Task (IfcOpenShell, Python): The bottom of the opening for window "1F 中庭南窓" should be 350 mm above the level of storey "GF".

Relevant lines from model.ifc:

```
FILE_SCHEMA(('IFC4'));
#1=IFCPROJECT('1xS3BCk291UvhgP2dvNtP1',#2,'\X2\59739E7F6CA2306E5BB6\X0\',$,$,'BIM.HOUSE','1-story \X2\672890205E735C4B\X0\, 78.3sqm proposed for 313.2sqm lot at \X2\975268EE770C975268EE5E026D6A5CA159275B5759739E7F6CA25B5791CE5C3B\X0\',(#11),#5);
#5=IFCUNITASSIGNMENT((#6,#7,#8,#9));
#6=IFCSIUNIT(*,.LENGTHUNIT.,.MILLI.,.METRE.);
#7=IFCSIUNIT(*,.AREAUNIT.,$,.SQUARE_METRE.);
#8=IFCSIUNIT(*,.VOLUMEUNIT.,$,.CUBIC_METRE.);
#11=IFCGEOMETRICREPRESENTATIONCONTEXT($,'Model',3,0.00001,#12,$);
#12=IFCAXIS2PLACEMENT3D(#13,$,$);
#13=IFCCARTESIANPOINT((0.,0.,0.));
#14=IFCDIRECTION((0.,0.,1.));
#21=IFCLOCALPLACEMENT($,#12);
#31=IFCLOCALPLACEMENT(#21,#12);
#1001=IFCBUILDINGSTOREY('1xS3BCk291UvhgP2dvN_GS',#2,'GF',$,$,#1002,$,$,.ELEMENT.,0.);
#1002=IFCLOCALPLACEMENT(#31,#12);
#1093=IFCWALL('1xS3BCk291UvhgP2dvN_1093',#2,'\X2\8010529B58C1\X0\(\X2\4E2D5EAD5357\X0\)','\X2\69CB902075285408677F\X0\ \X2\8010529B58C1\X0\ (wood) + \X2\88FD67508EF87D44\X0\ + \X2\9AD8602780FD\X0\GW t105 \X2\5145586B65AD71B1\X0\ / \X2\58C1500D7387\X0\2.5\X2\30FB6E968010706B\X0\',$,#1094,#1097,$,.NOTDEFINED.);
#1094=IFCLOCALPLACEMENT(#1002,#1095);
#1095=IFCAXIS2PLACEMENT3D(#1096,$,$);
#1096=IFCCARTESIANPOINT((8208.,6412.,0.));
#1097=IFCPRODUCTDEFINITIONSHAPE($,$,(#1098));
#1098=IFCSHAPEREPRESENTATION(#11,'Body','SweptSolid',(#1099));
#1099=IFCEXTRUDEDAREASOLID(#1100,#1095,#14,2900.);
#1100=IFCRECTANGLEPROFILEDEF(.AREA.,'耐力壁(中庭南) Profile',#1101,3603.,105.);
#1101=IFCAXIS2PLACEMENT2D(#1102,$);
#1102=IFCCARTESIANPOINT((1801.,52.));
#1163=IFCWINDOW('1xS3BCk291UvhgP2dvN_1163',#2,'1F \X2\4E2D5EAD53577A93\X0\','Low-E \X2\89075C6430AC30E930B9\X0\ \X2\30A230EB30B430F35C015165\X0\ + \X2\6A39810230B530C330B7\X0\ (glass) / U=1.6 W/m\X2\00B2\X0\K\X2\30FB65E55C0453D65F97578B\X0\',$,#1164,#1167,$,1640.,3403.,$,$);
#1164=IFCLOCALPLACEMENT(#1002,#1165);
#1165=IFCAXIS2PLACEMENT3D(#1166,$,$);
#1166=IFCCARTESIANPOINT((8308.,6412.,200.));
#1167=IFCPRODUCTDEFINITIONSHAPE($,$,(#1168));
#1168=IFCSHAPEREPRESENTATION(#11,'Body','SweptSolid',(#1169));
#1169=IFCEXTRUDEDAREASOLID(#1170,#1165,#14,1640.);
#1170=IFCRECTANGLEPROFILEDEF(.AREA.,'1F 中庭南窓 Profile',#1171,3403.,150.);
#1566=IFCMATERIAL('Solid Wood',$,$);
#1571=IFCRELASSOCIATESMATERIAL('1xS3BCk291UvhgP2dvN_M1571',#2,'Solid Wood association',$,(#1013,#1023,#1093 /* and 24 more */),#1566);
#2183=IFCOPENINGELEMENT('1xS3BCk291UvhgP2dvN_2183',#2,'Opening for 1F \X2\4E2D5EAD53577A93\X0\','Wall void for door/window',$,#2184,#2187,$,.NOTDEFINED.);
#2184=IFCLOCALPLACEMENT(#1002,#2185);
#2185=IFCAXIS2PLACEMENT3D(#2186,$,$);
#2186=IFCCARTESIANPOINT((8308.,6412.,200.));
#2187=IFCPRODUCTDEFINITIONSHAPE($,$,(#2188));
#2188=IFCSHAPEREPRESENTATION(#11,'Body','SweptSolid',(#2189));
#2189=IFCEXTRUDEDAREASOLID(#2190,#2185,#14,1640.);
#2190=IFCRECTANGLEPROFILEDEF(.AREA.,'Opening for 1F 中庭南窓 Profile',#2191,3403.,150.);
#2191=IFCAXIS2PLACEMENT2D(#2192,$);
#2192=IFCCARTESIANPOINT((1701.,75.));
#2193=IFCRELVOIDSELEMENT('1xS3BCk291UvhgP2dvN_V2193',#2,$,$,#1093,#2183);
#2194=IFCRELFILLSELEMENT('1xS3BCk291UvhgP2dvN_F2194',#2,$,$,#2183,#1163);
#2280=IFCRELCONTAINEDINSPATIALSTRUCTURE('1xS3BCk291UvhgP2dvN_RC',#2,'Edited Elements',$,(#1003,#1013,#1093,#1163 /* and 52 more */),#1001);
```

```python
import numpy as np
import ifcopenshell
import ifcopenshell.api.geometry
import ifcopenshell.geom
import ifcopenshell.util.element
import ifcopenshell.util.placement
import ifcopenshell.util.shape
import ifcopenshell.util.unit

model = ifcopenshell.open("model.ifc")
unit_scale = ifcopenshell.util.unit.calculate_unit_scale(model)

window = model.by_guid("1xS3BCk291UvhgP2dvN_1163")
opening = window.FillsVoids[0].RelatingOpeningElement
storey = ifcopenshell.util.element.get_container(window, ifc_class="IfcBuildingStorey")
level = ifcopenshell.util.placement.get_local_placement(storey.ObjectPlacement)[2, 3]

# The opening's origin need not be at the sill, so measure its lowest point.
shape = ifcopenshell.geom.create_shape(ifcopenshell.geom.settings(), opening)
bottom = ifcopenshell.util.shape.get_shape_bottom_elevation(shape, shape.geometry) / unit_scale
dz = level + 350.0 - bottom

shift = np.array([0.0, 0.0, dz])
# The window is not placed relative to its opening, so move both.
for product in (opening, window):
    matrix = ifcopenshell.util.placement.get_local_placement(product.ObjectPlacement)
    matrix[:3, 3] += shift
    ifcopenshell.api.geometry.edit_object_placement(model, product=product, matrix=matrix, is_si=False)

print(f"moved by {dz * unit_scale:+.3f} m")

model.write("model_v2.ifc")
```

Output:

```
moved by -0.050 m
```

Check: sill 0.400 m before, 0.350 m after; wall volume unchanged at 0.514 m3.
